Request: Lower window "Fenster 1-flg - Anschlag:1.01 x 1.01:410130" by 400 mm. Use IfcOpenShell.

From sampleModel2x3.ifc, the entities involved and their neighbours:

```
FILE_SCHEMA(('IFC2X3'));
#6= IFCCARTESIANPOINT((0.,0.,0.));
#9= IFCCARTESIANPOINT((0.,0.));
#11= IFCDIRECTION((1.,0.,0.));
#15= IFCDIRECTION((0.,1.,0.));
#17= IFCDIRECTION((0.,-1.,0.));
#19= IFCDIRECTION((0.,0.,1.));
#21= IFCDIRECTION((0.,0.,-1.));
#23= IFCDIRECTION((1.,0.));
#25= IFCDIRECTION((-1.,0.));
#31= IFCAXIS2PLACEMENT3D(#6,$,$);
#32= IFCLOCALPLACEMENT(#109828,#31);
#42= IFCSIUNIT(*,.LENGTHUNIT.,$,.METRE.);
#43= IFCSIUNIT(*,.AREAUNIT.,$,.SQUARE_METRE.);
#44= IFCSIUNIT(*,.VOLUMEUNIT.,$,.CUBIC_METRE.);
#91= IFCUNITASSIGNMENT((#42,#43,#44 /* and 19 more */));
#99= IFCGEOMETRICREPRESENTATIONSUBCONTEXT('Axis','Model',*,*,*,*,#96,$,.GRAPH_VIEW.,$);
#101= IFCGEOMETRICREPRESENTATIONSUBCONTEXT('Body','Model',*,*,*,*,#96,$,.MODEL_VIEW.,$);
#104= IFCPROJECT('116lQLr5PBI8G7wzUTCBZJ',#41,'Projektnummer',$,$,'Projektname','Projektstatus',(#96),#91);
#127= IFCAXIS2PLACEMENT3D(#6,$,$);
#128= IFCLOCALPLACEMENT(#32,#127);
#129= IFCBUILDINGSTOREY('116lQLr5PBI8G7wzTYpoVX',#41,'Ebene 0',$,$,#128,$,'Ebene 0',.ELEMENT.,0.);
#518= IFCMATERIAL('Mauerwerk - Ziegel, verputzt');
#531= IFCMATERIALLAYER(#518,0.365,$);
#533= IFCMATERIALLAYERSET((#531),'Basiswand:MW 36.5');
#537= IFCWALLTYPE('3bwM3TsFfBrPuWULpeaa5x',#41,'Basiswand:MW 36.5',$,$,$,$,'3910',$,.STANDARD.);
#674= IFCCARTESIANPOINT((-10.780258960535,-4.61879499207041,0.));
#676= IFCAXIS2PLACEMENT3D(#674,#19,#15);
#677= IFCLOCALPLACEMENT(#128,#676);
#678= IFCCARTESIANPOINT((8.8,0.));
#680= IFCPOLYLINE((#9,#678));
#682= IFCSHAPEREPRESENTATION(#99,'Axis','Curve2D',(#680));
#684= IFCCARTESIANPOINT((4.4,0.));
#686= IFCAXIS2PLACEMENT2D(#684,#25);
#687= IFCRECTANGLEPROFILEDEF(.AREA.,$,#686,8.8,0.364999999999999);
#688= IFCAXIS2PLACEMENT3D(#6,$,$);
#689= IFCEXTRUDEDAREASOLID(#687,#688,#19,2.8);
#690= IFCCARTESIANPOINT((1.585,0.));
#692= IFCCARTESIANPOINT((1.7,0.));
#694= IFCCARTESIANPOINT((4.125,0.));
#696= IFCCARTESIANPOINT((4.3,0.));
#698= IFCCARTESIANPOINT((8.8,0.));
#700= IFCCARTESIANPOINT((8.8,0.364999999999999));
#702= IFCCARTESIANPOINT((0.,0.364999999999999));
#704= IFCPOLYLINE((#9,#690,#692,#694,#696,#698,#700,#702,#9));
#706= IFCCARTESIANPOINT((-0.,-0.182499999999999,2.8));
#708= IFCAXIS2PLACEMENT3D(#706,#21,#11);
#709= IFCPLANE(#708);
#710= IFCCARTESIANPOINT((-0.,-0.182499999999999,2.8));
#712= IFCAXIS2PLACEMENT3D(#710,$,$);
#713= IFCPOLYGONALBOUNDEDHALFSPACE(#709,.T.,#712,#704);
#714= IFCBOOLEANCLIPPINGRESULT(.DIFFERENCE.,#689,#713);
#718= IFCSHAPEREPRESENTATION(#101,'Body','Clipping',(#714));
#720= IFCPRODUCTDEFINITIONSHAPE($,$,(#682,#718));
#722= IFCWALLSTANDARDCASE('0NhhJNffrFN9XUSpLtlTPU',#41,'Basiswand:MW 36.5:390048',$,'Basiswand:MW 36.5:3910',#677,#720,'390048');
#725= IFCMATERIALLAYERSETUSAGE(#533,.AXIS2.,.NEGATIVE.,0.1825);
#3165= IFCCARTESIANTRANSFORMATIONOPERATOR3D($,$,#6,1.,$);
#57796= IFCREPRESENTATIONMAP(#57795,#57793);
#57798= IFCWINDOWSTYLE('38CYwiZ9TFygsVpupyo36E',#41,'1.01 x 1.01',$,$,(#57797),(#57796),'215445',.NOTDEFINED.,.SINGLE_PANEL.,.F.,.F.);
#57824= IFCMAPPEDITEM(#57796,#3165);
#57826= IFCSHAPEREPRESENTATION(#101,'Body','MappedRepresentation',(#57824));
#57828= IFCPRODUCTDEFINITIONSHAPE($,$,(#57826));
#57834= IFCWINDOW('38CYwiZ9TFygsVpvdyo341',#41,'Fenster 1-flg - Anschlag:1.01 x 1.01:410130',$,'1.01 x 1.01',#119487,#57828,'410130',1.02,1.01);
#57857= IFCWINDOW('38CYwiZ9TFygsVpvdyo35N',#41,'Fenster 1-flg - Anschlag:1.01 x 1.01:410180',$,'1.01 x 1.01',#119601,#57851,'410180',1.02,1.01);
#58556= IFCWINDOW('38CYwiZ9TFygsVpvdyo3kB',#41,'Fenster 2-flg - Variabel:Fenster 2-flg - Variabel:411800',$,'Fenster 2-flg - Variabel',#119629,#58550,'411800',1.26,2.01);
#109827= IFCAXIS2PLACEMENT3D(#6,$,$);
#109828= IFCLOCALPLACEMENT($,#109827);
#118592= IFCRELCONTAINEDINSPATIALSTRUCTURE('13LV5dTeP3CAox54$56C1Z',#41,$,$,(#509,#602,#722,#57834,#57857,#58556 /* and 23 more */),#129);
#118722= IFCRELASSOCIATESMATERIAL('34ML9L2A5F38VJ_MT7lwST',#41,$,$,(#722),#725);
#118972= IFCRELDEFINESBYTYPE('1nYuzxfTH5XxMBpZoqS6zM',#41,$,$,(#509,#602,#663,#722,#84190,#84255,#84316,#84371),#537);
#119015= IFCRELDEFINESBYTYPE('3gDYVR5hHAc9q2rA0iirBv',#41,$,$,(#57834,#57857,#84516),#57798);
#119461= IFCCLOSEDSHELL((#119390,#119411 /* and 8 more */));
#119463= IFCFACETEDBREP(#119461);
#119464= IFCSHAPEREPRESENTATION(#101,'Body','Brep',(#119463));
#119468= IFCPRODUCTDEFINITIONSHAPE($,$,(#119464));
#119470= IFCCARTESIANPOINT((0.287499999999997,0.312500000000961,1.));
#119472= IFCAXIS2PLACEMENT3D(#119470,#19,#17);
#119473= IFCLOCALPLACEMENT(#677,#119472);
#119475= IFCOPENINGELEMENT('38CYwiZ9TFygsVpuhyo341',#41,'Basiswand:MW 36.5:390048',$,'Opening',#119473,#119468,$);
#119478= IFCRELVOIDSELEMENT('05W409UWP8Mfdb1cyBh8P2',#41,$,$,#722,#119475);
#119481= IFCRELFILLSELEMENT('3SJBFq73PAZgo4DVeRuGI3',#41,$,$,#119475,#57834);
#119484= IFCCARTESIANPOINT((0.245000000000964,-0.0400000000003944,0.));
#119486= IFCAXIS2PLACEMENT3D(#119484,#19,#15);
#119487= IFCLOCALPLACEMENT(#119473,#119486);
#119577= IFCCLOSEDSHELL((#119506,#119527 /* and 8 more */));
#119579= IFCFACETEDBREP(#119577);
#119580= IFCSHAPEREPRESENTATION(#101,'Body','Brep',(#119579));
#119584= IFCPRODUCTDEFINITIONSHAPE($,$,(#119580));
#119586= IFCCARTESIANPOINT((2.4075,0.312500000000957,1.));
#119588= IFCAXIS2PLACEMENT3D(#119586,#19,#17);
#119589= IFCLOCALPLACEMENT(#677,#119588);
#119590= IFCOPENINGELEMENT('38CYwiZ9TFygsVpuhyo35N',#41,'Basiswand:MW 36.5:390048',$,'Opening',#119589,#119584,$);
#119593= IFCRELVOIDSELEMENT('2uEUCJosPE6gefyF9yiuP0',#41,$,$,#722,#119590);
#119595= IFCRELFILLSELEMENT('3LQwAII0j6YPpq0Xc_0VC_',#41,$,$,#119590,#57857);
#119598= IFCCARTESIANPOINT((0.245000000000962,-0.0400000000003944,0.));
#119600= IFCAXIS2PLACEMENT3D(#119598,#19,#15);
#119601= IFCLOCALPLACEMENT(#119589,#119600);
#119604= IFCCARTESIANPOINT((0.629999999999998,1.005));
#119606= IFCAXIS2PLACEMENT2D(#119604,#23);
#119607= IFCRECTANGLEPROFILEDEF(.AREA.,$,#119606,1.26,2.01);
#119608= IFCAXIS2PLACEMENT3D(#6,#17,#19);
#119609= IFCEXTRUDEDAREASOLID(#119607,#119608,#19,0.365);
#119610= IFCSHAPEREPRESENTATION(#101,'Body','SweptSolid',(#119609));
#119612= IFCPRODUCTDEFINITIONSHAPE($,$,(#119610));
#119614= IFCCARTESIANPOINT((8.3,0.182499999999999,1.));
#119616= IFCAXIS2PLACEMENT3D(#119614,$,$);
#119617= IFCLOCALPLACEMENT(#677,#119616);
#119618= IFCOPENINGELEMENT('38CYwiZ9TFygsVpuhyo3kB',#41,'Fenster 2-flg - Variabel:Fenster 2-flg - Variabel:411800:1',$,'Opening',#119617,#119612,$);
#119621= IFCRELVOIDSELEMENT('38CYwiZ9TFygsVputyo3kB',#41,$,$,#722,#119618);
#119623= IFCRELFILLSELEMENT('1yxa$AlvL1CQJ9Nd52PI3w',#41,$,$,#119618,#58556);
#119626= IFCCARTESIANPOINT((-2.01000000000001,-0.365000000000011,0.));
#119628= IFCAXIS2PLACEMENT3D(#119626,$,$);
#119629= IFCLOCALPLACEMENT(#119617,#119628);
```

```python
import numpy as np
import ifcopenshell
import ifcopenshell.api.geometry
import ifcopenshell.util.placement
import ifcopenshell.util.unit

model = ifcopenshell.open("sampleModel2x3.ifc")
unit_scale = ifcopenshell.util.unit.calculate_unit_scale(model)

window = model.by_guid("38CYwiZ9TFygsVpvdyo341")
opening = window.FillsVoids[0].RelatingOpeningElement
dz = -0.4 / unit_scale

shift = np.array([0.0, 0.0, dz])
# The window is placed relative to its opening, so it follows when the opening moves.
matrix = ifcopenshell.util.placement.get_local_placement(opening.ObjectPlacement)
matrix[:3, 3] += shift
ifcopenshell.api.geometry.edit_object_placement(
    model, product=opening, matrix=matrix, is_si=False, should_transform_children=True
)

print(f"moved by {dz * unit_scale:+.3f} m")

model.write("sampleModel2x3_edited.ifc")
```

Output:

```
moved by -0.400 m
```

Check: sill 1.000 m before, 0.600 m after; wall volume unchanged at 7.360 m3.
